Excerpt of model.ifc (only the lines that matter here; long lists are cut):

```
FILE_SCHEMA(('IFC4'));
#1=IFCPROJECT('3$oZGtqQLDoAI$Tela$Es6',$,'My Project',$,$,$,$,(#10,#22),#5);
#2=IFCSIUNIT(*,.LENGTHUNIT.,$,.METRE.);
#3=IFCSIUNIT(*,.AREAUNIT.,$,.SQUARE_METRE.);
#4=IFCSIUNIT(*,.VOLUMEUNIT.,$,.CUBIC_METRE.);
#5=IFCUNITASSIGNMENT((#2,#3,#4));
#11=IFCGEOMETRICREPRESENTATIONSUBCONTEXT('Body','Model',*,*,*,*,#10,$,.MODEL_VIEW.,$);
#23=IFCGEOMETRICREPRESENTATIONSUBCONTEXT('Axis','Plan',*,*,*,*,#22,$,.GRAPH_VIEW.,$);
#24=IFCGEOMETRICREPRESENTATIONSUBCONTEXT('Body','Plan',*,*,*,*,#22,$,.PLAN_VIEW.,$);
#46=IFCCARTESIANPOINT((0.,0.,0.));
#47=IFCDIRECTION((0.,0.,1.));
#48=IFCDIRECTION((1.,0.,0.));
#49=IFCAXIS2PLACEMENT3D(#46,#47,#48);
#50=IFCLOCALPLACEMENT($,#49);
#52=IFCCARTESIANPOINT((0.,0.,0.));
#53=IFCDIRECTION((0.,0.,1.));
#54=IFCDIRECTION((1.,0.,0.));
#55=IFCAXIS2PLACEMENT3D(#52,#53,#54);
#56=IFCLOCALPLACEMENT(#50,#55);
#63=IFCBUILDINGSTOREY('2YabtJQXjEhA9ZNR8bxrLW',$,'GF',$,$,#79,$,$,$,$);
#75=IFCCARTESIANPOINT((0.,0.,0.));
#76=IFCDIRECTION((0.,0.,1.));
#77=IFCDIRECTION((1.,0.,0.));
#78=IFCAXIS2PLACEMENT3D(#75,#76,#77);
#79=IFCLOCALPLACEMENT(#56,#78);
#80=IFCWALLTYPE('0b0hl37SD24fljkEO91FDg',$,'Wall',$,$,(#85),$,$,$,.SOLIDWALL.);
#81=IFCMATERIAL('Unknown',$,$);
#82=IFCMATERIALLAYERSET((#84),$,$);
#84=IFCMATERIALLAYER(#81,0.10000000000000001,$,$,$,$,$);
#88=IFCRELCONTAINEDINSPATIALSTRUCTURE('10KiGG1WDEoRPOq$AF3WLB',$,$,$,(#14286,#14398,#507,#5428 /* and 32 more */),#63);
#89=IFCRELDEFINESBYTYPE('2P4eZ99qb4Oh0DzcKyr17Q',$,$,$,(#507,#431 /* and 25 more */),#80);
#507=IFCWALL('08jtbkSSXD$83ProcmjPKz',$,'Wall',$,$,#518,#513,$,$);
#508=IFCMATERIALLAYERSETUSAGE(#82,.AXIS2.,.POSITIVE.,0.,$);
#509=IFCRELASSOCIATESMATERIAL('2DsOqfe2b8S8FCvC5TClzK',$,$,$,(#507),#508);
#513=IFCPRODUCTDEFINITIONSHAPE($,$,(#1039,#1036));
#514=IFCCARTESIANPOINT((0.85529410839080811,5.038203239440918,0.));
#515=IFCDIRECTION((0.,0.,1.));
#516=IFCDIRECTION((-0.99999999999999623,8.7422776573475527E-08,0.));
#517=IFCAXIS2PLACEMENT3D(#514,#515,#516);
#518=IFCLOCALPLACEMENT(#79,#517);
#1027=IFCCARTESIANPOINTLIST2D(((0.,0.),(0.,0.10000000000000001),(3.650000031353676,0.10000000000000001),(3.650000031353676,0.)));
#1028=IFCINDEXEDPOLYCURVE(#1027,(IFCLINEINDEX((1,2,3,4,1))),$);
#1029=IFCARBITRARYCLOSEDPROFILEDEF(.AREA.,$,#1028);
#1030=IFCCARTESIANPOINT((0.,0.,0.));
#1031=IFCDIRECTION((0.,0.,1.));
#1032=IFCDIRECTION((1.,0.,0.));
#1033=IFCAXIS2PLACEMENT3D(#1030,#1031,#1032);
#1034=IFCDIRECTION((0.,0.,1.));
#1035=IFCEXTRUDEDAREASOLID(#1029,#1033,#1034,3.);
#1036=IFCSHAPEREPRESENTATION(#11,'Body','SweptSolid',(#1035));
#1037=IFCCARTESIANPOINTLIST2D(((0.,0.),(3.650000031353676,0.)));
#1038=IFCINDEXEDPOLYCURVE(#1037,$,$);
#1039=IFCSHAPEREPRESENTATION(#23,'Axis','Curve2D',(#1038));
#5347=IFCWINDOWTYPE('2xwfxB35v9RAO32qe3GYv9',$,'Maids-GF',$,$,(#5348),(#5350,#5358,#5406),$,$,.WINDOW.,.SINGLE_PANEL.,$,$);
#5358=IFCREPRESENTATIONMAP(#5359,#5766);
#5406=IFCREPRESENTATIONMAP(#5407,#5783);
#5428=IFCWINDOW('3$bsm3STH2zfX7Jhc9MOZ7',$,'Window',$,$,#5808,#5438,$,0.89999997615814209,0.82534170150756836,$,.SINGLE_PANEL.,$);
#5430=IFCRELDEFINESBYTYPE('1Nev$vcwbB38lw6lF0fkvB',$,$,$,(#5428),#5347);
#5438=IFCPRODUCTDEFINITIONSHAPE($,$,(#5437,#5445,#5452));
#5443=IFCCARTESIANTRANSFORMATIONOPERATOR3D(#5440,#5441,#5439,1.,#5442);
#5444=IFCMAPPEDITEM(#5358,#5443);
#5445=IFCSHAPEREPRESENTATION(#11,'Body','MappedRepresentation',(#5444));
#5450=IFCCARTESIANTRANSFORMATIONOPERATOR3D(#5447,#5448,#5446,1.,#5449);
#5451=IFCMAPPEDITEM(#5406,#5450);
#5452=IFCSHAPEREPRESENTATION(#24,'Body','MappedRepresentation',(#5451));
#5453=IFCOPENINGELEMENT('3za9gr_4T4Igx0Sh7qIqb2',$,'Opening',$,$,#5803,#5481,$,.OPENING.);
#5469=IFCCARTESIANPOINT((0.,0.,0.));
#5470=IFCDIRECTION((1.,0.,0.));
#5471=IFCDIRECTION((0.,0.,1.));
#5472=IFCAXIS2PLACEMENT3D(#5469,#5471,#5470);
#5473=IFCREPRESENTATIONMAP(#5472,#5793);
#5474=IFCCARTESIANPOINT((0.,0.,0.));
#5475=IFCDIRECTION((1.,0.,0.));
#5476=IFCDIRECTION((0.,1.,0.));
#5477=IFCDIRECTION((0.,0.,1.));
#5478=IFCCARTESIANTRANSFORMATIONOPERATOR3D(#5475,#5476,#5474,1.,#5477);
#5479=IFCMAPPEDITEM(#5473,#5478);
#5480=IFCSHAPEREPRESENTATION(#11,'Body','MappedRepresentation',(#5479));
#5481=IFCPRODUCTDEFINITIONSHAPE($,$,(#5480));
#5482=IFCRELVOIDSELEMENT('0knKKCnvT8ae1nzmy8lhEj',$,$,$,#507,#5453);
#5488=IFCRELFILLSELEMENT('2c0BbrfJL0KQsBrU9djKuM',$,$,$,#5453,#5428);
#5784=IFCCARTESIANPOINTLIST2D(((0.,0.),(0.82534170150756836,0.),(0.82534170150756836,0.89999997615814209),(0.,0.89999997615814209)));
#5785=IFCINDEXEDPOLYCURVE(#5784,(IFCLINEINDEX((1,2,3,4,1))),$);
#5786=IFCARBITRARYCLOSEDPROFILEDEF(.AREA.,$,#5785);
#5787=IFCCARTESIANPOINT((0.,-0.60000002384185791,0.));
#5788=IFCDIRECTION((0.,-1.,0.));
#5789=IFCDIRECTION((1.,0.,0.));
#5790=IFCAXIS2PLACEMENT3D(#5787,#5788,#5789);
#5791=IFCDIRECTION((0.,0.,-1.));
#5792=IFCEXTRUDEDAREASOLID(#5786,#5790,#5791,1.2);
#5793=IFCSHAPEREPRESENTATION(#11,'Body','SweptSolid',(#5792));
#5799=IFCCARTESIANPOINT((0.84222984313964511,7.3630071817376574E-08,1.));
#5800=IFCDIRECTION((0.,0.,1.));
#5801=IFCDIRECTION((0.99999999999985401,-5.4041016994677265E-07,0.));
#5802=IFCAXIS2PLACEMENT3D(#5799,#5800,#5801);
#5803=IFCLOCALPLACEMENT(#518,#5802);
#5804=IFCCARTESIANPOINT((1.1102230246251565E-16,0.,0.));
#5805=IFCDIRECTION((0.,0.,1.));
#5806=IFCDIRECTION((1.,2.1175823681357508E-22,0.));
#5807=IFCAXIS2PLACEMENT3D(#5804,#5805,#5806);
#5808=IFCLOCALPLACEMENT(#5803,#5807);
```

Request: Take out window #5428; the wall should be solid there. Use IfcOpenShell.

```python
import ifcopenshell
import ifcopenshell.api.feature
import ifcopenshell.api.root
import ifcopenshell.geom
import ifcopenshell.util.shape

model = ifcopenshell.open("model.ifc")
settings = ifcopenshell.geom.settings()


def volume(element):
    """Net volume in cubic metres, openings subtracted."""
    shape = ifcopenshell.geom.create_shape(settings, element)
    return ifcopenshell.util.shape.get_volume(shape.geometry)


window = model.by_id(5428)
opening = window.FillsVoids[0].RelatingOpeningElement
wall = opening.VoidsElements[0].RelatingBuildingElement
before = volume(wall)

ifcopenshell.api.root.remove_product(model, product=window)
ifcopenshell.api.feature.remove_feature(model, feature=opening)

after = volume(wall)

print(f"wall volume {before:.3f} -> {after:.3f} m3")

model.write("model_edited.ifc")
```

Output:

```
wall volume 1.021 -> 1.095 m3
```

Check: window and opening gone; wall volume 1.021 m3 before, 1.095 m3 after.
